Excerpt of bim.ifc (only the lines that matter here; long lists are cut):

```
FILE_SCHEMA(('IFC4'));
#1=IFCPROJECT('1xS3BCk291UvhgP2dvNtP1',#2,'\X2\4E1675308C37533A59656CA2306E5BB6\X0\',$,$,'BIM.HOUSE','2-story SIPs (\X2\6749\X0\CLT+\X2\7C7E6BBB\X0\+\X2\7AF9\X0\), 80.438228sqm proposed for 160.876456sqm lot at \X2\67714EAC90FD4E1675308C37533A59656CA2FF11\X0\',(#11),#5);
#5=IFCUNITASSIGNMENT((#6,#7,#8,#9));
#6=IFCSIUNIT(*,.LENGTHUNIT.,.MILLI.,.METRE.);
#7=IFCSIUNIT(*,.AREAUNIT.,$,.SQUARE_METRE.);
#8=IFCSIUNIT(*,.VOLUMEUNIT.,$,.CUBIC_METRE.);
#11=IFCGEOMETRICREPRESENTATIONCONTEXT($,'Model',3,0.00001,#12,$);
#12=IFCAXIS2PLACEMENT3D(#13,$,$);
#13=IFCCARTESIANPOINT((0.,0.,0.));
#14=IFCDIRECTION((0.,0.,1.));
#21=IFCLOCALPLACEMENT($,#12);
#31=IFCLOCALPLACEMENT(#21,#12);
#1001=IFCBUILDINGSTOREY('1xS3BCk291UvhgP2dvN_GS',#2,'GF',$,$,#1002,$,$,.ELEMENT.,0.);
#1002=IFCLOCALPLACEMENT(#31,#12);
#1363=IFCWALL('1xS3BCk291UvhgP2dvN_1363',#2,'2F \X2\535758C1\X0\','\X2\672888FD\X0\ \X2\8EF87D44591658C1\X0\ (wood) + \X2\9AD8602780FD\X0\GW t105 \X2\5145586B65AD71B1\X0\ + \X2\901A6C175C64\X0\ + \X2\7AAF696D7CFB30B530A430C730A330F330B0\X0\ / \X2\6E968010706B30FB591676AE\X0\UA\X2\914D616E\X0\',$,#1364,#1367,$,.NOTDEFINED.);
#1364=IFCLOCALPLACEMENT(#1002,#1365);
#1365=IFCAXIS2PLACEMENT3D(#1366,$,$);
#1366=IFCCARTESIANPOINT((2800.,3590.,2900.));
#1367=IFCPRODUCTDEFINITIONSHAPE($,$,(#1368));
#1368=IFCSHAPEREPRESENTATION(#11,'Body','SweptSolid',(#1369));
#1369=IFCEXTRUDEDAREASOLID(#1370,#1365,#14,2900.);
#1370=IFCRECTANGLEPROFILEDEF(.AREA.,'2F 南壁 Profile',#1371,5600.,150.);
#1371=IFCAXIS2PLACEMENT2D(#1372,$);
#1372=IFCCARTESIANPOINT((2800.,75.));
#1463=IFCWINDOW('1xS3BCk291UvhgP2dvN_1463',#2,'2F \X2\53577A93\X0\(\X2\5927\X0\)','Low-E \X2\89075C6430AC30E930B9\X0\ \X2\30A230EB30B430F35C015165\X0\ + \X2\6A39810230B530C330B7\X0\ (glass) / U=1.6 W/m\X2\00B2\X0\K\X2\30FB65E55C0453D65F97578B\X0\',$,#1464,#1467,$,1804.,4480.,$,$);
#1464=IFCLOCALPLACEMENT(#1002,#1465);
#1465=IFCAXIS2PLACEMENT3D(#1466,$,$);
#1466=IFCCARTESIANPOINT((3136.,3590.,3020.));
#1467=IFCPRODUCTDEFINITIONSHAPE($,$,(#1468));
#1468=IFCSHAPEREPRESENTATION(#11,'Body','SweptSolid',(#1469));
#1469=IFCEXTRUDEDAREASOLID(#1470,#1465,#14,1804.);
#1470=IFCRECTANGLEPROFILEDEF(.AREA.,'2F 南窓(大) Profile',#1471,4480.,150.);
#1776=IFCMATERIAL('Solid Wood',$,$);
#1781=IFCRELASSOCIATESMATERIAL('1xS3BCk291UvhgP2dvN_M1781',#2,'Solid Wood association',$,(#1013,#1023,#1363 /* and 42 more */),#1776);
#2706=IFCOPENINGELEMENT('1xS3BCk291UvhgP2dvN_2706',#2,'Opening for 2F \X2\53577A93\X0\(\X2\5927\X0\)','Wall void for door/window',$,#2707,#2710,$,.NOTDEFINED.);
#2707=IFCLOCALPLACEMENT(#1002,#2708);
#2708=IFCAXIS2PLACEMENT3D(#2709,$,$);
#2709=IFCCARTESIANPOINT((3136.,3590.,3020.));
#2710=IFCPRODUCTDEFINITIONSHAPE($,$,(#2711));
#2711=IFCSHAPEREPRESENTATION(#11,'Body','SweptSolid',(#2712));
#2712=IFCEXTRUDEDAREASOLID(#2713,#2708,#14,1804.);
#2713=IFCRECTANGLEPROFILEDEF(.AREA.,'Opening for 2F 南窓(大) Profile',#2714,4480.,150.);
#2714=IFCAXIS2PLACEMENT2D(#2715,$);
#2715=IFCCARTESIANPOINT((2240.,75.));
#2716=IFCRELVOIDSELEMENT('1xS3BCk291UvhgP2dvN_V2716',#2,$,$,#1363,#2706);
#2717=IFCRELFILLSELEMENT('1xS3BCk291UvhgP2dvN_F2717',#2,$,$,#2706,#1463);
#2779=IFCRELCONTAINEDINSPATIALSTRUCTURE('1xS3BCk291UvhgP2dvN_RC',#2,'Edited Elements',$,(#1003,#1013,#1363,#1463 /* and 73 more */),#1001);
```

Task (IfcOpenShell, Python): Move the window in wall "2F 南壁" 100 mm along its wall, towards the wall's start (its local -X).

```python
import ifcopenshell
import ifcopenshell.api.geometry
import ifcopenshell.util.placement
import ifcopenshell.util.unit

model = ifcopenshell.open("bim.ifc")
unit_scale = ifcopenshell.util.unit.calculate_unit_scale(model)

window = model.by_id(1463)
opening = window.FillsVoids[0].RelatingOpeningElement
wall = opening.VoidsElements[0].RelatingBuildingElement

wall_matrix = ifcopenshell.util.placement.get_local_placement(wall.ObjectPlacement)
shift = wall_matrix[:3, 0] * -0.1 / unit_scale
before = ifcopenshell.util.placement.get_local_placement(window.ObjectPlacement)[:3, 3].copy()

# The window is not placed relative to its opening, so move both.
for product in (opening, window):
    matrix = ifcopenshell.util.placement.get_local_placement(product.ObjectPlacement)
    matrix[:3, 3] += shift
    ifcopenshell.api.geometry.edit_object_placement(model, product=product, matrix=matrix, is_si=False)

after = ifcopenshell.util.placement.get_local_placement(window.ObjectPlacement)[:3, 3]
print("window moved by", (after - before).round(3) + 0.0)

model.write("bim-out.ifc")
```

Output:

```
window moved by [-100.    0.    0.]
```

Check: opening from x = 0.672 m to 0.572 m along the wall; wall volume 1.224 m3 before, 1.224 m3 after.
